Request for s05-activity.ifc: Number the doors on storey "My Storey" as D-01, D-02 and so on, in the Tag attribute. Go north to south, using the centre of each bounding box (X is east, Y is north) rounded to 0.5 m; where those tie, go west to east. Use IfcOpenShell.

First a look at what the model holds.

```python
import ifcopenshell
import ifcopenshell.util.element
import ifcopenshell.util.placement

model = ifcopenshell.open("s05-activity.ifc")
print(model.schema)
storey = next(s for s in model.by_type("IfcBuildingStorey") if s.Name == "My Storey")
doors = [e for e in ifcopenshell.util.element.get_decomposition(storey) if e.is_a("IfcDoor")]
for e in sorted(doors, key=lambda e: e.id()):
    origin = ifcopenshell.util.placement.get_local_placement(e.ObjectPlacement)[:3, 3]
    print(e.id(), e.Tag, e.Name, origin.round(2) + 0.0, sep=" | ")
```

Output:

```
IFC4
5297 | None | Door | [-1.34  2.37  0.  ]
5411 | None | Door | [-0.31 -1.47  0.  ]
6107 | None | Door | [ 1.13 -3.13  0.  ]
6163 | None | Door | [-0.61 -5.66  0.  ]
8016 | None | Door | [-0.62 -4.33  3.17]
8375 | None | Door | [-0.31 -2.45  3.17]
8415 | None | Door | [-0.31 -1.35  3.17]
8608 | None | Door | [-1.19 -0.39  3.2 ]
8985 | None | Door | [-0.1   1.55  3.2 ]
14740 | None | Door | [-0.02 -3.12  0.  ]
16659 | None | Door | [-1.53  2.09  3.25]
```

```python
import ifcopenshell
import ifcopenshell.geom
import ifcopenshell.util.element
import ifcopenshell.util.shape

model = ifcopenshell.open("s05-activity.ifc")
settings = ifcopenshell.geom.settings()
settings.set("use-world-coords", True)


def centre(element):
    shape = ifcopenshell.geom.create_shape(settings, element)
    return ifcopenshell.util.shape.get_bbox_centroid(shape.geometry)


storey = next(s for s in model.by_type("IfcBuildingStorey") if s.Name == "My Storey")
doors = [e for e in ifcopenshell.util.element.get_decomposition(storey) if e.is_a("IfcDoor")]

# Insertion points can sit at a corner or the storey origin, so sort by the geometry (in metres).
centres = {e: centre(e) for e in doors}
doors.sort(key=lambda e: (-round(centres[e][1] / 0.5), centres[e][0]))

for i, e in enumerate(doors, start=1):
    number = f"D-{i:02d}"
    e.Tag = number
    print(e.id(), number)

model.write("s05-activity_edited.ifc")
```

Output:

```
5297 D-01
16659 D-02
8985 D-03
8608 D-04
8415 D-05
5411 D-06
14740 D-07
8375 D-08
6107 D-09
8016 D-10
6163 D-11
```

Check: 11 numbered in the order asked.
